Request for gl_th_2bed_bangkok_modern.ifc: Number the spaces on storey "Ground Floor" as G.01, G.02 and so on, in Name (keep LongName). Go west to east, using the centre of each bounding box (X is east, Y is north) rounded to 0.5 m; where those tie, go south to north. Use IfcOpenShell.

First a look at what the model holds.

```python
import ifcopenshell
import ifcopenshell.util.element
import ifcopenshell.util.placement

model = ifcopenshell.open("gl_th_2bed_bangkok_modern.ifc")
print(model.schema)
storey = next(s for s in model.by_type("IfcBuildingStorey") if s.Name == "Ground Floor")
spaces = [e for e in ifcopenshell.util.element.get_decomposition(storey) if e.is_a("IfcSpace")]
for e in sorted(spaces, key=lambda e: e.id()):
    origin = ifcopenshell.util.placement.get_local_placement(e.ObjectPlacement)[:3, 3]
    print(e.id(), e.Name, e.LongName, origin.round(2) + 0.0, sep=" | ")
```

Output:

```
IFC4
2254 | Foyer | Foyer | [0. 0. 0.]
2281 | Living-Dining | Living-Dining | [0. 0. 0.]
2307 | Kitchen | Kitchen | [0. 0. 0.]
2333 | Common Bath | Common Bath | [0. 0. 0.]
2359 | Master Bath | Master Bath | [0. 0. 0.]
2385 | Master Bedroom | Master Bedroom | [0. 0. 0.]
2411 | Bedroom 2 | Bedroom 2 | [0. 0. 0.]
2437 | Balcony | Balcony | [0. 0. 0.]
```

```python
import ifcopenshell
import ifcopenshell.geom
import ifcopenshell.util.element
import ifcopenshell.util.shape

model = ifcopenshell.open("gl_th_2bed_bangkok_modern.ifc")
settings = ifcopenshell.geom.settings()
settings.set("use-world-coords", True)


def centre(element):
    shape = ifcopenshell.geom.create_shape(settings, element)
    return ifcopenshell.util.shape.get_bbox_centroid(shape.geometry)


storey = next(s for s in model.by_type("IfcBuildingStorey") if s.Name == "Ground Floor")
spaces = [e for e in ifcopenshell.util.element.get_decomposition(storey) if e.is_a("IfcSpace")]

# Insertion points can sit at a corner or the storey origin, so sort by the geometry (in metres).
centres = {e: centre(e) for e in spaces}
spaces.sort(key=lambda e: (round(centres[e][0] / 0.5), centres[e][1]))

for i, e in enumerate(spaces, start=1):
    number = f"G.{i:02d}"
    e.Name = number
    print(e.id(), number)

model.write("gl_th_2bed_bangkok_modern_rev.ifc")
```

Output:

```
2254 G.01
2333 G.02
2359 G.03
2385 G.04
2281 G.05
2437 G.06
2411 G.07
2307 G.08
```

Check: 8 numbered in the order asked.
